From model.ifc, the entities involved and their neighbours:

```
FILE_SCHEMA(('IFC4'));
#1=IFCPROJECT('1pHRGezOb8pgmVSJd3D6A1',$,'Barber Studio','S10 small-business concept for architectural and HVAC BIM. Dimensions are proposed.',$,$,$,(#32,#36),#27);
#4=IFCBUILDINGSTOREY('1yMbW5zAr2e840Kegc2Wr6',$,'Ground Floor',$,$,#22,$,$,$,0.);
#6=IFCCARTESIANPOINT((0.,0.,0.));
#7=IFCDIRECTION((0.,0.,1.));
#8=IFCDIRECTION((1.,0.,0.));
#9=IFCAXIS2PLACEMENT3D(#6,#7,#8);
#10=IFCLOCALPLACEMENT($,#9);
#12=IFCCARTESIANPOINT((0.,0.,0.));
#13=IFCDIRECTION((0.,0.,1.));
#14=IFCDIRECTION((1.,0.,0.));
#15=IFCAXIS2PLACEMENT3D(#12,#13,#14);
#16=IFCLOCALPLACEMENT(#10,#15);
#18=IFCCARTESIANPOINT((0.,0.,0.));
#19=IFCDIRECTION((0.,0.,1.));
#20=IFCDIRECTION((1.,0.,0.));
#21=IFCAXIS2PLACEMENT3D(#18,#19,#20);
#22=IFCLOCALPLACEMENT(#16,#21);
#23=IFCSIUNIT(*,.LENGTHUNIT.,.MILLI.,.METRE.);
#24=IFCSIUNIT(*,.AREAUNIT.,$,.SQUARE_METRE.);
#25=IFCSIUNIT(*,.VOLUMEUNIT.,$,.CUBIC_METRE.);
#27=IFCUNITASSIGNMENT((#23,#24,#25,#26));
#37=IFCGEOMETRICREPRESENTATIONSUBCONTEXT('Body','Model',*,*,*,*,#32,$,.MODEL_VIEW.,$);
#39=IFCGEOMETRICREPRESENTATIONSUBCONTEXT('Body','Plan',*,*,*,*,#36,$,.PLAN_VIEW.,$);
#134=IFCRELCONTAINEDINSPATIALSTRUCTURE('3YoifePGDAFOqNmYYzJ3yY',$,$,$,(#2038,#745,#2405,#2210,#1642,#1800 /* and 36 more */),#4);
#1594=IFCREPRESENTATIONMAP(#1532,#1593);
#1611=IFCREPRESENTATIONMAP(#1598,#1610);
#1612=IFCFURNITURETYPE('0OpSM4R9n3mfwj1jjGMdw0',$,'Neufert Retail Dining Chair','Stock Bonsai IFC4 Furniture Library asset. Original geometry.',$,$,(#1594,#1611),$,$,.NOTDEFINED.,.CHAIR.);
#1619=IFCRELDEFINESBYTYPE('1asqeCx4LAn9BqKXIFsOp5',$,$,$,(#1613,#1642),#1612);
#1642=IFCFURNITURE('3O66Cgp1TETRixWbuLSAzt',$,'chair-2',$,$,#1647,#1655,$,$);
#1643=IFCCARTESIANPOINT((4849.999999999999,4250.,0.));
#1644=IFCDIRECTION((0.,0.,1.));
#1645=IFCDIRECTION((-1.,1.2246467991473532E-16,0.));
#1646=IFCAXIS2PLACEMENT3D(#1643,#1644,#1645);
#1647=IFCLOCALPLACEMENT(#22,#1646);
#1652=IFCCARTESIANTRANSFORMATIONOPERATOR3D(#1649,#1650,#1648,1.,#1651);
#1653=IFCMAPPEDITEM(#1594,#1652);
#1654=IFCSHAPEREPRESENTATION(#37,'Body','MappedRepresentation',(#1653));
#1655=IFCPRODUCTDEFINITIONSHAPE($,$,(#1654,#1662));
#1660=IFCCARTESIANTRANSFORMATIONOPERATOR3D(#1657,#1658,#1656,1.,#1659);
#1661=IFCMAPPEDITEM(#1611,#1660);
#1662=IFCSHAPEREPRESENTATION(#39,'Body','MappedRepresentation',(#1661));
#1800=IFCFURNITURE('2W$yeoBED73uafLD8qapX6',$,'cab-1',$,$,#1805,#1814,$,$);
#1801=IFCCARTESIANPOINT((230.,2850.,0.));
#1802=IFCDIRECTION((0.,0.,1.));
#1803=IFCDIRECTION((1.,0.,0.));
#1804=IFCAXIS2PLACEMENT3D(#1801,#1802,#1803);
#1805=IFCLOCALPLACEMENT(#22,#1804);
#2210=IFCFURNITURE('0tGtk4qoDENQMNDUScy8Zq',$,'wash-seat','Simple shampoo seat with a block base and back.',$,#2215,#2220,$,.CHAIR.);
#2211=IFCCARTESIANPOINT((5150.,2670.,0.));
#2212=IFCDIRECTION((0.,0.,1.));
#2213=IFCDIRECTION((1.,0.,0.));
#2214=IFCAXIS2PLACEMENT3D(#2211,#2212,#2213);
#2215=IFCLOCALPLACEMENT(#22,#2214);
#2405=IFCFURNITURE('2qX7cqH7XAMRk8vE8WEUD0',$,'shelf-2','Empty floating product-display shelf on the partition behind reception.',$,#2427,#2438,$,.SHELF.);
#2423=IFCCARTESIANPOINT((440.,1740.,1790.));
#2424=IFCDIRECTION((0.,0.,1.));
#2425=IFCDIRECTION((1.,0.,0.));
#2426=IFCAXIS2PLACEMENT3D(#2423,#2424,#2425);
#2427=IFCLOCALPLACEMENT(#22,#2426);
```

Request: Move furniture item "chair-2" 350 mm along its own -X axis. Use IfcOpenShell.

```python
import ifcopenshell
import ifcopenshell.api.geometry
import ifcopenshell.util.placement
import ifcopenshell.util.unit

model = ifcopenshell.open("model.ifc")
unit_scale = ifcopenshell.util.unit.calculate_unit_scale(model)

item = model.by_guid("3O66Cgp1TETRixWbuLSAzt")
matrix = ifcopenshell.util.placement.get_local_placement(item.ObjectPlacement)
matrix[:3, 3] -= matrix[:3, 0] * 0.35 / unit_scale
ifcopenshell.api.geometry.edit_object_placement(model, product=item, matrix=matrix, is_si=False)

print(ifcopenshell.util.placement.get_local_placement(item.ObjectPlacement).round(3) + 0.0)

model.write("model_updated.ifc")
```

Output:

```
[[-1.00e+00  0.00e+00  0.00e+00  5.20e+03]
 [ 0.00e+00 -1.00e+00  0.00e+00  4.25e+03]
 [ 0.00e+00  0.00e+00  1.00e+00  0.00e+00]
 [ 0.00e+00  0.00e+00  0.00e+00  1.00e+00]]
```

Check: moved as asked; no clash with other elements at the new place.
